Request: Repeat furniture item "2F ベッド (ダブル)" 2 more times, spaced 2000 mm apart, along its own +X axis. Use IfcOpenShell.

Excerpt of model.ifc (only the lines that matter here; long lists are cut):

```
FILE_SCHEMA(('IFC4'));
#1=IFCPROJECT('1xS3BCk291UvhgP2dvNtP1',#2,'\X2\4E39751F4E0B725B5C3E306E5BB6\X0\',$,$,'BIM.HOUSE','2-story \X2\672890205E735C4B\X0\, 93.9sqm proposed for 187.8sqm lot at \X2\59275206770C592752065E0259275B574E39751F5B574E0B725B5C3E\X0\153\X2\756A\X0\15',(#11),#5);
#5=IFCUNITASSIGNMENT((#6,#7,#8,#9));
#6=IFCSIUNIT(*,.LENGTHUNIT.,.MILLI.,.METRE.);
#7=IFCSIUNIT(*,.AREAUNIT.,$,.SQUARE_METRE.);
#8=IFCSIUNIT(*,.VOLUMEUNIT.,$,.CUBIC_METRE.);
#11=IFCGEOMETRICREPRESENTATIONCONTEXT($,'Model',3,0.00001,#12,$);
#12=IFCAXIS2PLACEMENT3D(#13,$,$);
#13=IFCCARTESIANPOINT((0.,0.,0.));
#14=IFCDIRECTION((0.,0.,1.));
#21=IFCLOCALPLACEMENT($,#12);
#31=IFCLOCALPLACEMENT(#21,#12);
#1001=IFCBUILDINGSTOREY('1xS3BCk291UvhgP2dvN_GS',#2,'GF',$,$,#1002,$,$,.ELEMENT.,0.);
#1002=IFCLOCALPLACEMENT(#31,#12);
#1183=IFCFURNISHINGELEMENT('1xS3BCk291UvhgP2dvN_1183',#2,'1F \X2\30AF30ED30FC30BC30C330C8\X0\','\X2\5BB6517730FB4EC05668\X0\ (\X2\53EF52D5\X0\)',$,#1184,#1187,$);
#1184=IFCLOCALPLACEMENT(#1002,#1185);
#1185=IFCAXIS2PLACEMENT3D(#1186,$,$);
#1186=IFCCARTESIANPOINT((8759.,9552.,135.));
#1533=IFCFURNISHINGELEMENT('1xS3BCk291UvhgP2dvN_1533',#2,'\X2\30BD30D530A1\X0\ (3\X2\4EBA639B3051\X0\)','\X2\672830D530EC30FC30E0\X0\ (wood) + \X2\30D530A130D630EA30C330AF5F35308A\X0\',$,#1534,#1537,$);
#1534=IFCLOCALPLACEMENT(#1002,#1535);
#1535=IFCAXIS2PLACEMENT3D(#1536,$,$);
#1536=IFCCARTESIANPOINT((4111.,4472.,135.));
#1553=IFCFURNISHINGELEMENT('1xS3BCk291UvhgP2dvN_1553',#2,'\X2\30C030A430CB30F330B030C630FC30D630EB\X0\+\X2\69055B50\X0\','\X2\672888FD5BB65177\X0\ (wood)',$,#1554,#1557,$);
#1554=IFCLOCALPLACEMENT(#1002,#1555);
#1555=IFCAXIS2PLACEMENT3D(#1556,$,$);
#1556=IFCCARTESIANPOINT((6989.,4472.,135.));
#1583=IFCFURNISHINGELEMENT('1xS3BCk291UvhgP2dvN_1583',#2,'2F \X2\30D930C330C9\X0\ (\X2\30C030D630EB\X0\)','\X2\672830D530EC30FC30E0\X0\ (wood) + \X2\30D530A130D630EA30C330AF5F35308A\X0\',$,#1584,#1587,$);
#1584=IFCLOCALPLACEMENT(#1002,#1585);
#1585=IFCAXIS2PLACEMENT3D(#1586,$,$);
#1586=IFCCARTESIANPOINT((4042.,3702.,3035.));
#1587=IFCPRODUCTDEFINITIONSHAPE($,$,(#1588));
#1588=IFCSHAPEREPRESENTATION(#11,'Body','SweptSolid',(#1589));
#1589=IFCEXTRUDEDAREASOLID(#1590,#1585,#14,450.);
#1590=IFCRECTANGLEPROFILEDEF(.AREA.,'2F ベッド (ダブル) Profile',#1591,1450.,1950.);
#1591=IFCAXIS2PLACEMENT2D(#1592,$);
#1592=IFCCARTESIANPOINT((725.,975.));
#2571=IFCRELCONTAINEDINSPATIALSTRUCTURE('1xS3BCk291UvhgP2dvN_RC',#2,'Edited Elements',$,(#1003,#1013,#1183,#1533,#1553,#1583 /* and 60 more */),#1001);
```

```python
import ifcopenshell
import ifcopenshell.api.geometry
import ifcopenshell.api.root
import ifcopenshell.util.element
import ifcopenshell.util.placement
import ifcopenshell.util.unit

model = ifcopenshell.open("model.ifc")
unit_scale = ifcopenshell.util.unit.calculate_unit_scale(model)


def reuse_history(source, copy):
    """copy_class also copies each property set's owner history, people and application; keep the originals."""
    for rel in copy.IsDefinedBy:
        if rel.is_a("IfcRelDefinesByProperties") and (history := rel.RelatingPropertyDefinition.OwnerHistory):
            rel.RelatingPropertyDefinition.OwnerHistory = source.OwnerHistory
            ifcopenshell.util.element.remove_deep2(model, history)


source = model.by_guid("1xS3BCk291UvhgP2dvN_1583")
base = ifcopenshell.util.placement.get_local_placement(source.ObjectPlacement)
step = base[:3, 0] * 2 / unit_scale

for i in range(1, 3):
    copy = ifcopenshell.api.root.copy_class(model, product=source)
    copy.Representation = ifcopenshell.util.element.copy_deep(
        model, source.Representation, exclude=["IfcGeometricRepresentationContext", "IfcRepresentationMap"]
    )
    reuse_history(source, copy)
    matrix = base.copy()
    matrix[:3, 3] += i * step
    print("added at", matrix[:3, 3].round(3) + 0.0)
    ifcopenshell.api.geometry.edit_object_placement(model, product=copy, matrix=matrix, is_si=False)

model.write("model_edited.ifc")
```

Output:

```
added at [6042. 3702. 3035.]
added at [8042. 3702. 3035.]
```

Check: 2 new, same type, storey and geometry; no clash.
